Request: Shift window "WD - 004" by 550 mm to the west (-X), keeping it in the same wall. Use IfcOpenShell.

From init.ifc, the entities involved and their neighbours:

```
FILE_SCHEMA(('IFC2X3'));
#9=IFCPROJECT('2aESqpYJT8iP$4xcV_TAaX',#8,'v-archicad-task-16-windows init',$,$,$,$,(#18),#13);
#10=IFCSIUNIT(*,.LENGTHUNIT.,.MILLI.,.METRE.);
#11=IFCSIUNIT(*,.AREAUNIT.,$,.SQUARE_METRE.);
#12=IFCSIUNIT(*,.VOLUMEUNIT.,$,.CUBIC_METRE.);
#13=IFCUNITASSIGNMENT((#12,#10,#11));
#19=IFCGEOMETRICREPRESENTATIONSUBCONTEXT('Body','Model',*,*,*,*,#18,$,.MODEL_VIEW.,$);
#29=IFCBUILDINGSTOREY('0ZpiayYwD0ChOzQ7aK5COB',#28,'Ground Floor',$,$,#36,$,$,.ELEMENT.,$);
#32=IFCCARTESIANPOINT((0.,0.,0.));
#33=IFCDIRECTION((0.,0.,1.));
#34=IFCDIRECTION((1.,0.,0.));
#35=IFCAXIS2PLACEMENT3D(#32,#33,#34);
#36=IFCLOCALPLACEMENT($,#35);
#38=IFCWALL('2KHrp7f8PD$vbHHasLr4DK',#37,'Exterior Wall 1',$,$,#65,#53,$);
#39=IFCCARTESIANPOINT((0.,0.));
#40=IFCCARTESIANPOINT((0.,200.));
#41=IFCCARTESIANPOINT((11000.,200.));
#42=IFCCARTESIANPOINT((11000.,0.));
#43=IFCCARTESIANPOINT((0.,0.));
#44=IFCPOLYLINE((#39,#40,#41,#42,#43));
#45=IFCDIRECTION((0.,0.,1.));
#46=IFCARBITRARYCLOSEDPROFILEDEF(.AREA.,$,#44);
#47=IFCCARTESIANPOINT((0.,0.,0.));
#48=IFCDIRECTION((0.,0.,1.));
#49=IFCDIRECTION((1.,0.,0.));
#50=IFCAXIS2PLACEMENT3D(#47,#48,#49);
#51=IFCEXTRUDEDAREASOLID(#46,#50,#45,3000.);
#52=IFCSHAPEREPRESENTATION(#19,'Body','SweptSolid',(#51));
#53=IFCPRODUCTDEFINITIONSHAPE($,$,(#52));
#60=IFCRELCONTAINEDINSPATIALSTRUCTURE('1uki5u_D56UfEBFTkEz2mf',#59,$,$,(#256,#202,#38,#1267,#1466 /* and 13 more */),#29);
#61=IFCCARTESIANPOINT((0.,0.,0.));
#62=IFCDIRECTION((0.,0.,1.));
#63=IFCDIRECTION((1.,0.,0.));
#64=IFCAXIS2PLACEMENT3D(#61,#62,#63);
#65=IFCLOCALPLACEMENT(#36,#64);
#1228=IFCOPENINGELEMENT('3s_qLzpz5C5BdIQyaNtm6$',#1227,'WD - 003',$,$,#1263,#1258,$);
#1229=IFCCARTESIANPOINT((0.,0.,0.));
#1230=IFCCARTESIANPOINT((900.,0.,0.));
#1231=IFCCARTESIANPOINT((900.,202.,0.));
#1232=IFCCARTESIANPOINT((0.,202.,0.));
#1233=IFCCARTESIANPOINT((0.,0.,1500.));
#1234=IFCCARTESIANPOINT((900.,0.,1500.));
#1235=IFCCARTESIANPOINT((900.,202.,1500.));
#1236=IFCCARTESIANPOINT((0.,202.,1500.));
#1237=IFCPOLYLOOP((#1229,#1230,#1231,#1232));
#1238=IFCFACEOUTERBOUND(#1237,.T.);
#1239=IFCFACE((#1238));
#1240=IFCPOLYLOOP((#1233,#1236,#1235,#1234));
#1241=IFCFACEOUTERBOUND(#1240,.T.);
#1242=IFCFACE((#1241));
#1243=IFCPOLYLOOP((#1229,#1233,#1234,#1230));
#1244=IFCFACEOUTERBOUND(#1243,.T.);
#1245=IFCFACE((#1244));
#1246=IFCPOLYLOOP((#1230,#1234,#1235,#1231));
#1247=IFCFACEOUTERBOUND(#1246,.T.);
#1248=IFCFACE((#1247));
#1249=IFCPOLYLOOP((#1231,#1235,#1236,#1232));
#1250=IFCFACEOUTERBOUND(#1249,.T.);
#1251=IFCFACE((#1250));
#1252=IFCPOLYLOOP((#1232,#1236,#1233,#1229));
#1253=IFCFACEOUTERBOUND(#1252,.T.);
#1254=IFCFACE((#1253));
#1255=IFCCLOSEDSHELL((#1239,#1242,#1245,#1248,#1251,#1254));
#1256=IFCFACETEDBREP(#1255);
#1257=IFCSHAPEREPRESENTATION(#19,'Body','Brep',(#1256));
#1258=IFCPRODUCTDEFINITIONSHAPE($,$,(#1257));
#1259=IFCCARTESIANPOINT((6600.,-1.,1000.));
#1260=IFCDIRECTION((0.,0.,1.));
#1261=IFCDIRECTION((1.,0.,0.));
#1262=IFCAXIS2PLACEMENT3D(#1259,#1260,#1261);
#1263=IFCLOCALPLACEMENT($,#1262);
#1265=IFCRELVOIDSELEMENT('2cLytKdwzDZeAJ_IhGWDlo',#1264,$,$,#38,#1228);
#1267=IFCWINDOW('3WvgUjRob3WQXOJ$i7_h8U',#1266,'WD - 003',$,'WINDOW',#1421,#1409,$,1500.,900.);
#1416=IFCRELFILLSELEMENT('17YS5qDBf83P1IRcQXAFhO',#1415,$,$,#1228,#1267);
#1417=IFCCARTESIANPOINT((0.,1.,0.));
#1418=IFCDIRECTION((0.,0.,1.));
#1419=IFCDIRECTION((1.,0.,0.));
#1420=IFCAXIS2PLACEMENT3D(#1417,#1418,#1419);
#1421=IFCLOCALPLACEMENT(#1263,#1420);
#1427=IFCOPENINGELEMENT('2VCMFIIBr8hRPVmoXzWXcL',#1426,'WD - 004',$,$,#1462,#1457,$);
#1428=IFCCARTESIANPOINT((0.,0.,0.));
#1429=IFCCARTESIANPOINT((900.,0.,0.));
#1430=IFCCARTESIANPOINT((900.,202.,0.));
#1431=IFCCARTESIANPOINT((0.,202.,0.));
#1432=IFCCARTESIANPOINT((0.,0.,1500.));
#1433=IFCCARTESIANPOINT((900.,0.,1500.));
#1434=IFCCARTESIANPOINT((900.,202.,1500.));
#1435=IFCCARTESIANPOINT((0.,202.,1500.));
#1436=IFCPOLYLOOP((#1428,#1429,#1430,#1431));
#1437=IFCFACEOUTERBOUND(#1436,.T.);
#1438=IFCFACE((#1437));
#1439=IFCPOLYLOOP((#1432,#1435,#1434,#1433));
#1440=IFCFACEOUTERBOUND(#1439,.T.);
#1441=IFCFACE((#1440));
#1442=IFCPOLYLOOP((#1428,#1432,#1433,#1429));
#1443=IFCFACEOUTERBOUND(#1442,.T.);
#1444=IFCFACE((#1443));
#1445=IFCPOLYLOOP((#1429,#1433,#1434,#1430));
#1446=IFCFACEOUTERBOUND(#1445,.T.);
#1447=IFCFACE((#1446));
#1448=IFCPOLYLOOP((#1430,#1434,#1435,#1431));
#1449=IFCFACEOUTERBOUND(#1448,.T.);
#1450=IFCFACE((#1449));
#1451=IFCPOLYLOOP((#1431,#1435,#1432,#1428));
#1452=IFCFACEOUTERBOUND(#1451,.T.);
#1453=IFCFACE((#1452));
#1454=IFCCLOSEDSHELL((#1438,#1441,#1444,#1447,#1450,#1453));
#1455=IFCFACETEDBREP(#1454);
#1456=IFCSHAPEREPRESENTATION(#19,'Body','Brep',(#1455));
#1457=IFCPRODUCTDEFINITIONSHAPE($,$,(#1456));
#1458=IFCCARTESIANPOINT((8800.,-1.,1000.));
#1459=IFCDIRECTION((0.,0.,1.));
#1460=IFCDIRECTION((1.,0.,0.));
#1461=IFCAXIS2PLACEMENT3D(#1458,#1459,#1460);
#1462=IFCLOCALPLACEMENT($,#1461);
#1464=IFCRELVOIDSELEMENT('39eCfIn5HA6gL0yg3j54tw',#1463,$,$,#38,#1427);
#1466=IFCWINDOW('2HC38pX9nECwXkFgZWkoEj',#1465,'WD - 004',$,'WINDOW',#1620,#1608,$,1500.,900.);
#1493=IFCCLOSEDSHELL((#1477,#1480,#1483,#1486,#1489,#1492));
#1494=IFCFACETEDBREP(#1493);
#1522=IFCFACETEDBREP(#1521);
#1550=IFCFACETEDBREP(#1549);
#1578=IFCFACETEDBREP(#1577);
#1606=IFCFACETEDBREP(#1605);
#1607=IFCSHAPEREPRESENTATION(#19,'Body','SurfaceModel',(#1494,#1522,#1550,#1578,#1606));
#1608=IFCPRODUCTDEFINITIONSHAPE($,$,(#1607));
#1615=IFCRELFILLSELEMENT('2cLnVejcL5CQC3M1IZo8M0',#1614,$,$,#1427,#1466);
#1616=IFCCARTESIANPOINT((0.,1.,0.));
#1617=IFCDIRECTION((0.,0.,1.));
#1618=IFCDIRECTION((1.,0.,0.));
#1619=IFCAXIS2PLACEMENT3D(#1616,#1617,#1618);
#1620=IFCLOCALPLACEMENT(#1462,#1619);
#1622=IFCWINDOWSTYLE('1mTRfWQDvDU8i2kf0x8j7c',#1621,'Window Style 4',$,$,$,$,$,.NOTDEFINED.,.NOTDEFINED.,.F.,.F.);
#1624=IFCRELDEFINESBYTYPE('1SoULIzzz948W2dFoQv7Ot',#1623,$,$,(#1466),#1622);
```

```python
import ifcopenshell
import ifcopenshell.api.geometry
import ifcopenshell.util.placement
import ifcopenshell.util.unit

model = ifcopenshell.open("init.ifc")
unit_scale = ifcopenshell.util.unit.calculate_unit_scale(model)

window = model.by_guid("2HC38pX9nECwXkFgZWkoEj")
opening = window.FillsVoids[0].RelatingOpeningElement
wall = opening.VoidsElements[0].RelatingBuildingElement

wall_matrix = ifcopenshell.util.placement.get_local_placement(wall.ObjectPlacement)
shift = wall_matrix[:3, 0] * -0.55 / unit_scale
before = ifcopenshell.util.placement.get_local_placement(window.ObjectPlacement)[:3, 3].copy()

# The window is placed relative to its opening, so it follows when the opening moves.
matrix = ifcopenshell.util.placement.get_local_placement(opening.ObjectPlacement)
matrix[:3, 3] += shift
ifcopenshell.api.geometry.edit_object_placement(
    model, product=opening, matrix=matrix, is_si=False, should_transform_children=True
)

after = ifcopenshell.util.placement.get_local_placement(window.ObjectPlacement)[:3, 3]
print("window moved by", (after - before).round(3) + 0.0)

model.write("init-out.ifc")
```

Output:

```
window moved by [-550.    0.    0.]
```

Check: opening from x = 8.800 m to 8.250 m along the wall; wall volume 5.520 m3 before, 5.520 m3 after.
